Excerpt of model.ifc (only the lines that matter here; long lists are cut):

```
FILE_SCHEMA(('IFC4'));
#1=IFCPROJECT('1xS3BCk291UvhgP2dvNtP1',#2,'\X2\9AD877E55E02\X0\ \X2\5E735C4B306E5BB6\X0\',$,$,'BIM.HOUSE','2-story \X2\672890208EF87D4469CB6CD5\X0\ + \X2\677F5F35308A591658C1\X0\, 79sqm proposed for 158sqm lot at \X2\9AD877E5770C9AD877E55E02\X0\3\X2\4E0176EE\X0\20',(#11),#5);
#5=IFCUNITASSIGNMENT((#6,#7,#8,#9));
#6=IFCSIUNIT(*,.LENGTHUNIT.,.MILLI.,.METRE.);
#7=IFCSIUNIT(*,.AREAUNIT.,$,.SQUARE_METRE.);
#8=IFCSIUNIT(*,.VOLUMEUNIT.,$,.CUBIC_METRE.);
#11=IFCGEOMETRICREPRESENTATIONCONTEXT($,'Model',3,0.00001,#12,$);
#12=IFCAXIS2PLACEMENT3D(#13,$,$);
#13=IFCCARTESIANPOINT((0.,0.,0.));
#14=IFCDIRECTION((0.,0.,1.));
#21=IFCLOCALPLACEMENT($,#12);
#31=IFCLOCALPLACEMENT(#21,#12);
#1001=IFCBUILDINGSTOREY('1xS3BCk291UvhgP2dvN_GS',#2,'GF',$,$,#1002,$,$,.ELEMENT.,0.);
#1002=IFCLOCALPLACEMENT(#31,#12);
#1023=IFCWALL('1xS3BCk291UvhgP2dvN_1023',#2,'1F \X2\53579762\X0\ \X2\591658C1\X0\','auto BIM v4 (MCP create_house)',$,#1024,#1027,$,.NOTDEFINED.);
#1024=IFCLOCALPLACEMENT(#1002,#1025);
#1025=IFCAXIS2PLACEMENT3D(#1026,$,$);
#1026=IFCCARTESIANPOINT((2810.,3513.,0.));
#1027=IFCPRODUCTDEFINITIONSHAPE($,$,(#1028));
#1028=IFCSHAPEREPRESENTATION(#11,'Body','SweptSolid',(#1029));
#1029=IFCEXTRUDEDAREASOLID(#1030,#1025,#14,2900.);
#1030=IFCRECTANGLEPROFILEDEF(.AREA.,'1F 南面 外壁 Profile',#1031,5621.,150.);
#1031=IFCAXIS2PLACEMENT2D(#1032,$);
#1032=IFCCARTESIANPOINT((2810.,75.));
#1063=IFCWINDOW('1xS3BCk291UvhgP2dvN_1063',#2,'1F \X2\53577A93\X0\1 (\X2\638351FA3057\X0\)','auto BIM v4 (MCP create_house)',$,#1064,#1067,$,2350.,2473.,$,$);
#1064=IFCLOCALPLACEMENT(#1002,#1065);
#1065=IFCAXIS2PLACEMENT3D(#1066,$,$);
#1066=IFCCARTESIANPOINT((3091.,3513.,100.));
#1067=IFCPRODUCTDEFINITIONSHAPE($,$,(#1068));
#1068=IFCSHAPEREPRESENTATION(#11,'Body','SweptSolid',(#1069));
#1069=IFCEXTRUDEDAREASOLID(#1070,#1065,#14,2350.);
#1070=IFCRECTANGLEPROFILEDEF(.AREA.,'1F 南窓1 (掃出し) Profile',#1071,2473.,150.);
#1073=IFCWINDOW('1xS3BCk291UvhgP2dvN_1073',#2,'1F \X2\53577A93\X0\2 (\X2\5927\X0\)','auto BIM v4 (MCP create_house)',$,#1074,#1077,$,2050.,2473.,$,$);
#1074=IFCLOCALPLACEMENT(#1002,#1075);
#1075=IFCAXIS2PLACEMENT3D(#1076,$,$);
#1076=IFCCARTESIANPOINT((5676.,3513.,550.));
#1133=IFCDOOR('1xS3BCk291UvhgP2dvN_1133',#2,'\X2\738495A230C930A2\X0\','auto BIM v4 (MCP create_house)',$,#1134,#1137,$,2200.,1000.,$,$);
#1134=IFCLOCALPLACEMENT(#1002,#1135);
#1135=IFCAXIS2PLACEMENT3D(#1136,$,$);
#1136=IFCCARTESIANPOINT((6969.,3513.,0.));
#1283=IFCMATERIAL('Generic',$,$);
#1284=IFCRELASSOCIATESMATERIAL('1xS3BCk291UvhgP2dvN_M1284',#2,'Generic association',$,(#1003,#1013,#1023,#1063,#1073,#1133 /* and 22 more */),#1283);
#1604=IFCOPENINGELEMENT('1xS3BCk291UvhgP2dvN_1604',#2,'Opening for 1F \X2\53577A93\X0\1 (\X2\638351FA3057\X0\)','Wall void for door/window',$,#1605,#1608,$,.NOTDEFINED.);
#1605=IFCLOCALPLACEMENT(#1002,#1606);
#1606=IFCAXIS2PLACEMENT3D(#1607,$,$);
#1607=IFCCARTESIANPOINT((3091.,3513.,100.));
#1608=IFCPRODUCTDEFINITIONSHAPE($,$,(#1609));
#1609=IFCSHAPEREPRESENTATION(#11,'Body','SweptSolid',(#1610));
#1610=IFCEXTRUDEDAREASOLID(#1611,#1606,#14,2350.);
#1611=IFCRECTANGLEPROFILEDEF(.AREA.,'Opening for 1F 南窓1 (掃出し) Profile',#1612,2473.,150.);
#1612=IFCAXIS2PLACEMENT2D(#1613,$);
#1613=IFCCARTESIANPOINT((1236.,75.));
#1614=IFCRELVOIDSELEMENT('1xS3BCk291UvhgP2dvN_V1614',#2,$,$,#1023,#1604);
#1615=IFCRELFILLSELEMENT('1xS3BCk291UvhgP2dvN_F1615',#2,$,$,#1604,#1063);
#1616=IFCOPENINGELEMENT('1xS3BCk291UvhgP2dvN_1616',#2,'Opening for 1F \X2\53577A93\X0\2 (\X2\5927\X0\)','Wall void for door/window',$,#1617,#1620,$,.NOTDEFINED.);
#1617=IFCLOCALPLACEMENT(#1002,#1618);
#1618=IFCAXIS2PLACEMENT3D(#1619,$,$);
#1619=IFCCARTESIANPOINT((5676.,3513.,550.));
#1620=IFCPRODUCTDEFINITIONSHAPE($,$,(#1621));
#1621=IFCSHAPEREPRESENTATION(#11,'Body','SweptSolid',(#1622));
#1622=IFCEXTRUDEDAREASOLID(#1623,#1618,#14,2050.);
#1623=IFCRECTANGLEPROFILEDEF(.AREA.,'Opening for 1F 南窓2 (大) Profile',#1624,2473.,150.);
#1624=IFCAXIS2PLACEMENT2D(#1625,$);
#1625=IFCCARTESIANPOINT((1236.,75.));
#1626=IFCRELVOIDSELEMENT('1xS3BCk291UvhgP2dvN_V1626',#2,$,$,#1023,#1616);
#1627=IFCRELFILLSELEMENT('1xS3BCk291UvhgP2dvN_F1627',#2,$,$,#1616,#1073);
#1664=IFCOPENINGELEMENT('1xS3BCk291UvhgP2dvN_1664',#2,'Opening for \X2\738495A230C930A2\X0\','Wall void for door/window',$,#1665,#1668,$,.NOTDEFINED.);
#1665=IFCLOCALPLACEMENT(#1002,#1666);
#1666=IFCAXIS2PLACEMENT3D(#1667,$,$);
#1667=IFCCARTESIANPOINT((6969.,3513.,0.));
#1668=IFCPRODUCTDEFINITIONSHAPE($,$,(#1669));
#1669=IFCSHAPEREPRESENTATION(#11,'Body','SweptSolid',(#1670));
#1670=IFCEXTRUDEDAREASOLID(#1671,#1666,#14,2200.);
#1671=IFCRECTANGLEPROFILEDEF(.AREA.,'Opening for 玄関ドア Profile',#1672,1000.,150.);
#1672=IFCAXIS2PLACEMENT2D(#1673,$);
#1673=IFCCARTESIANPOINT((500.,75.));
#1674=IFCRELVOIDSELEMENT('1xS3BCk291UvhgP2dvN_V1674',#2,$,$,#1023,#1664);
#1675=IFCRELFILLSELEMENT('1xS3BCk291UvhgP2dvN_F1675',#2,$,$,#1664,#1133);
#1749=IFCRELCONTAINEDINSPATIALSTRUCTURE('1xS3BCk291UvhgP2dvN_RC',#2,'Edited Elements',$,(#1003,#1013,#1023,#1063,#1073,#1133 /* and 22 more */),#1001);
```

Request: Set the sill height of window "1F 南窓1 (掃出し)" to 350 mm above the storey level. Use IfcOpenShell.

```python
import numpy as np
import ifcopenshell
import ifcopenshell.api.geometry
import ifcopenshell.geom
import ifcopenshell.util.element
import ifcopenshell.util.placement
import ifcopenshell.util.shape
import ifcopenshell.util.unit

model = ifcopenshell.open("model.ifc")
unit_scale = ifcopenshell.util.unit.calculate_unit_scale(model)

window = model.by_guid("1xS3BCk291UvhgP2dvN_1063")
opening = window.FillsVoids[0].RelatingOpeningElement
storey = ifcopenshell.util.element.get_container(window, ifc_class="IfcBuildingStorey")
level = ifcopenshell.util.placement.get_local_placement(storey.ObjectPlacement)[2, 3]

# The opening's origin need not be at the sill, so measure its lowest point.
shape = ifcopenshell.geom.create_shape(ifcopenshell.geom.settings(), opening)
bottom = ifcopenshell.util.shape.get_shape_bottom_elevation(shape, shape.geometry) / unit_scale
dz = level + 350.0 - bottom

shift = np.array([0.0, 0.0, dz])
# The window is not placed relative to its opening, so move both.
for product in (opening, window):
    matrix = ifcopenshell.util.placement.get_local_placement(product.ObjectPlacement)
    matrix[:3, 3] += shift
    ifcopenshell.api.geometry.edit_object_placement(model, product=product, matrix=matrix, is_si=False)

print(f"moved by {dz * unit_scale:+.3f} m")

model.write("model-out.ifc")
```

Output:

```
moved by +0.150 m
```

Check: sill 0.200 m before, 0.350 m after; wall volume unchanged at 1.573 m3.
